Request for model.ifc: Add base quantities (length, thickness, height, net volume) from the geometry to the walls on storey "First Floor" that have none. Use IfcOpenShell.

First a look at what the model holds.

```python
import ifcopenshell
import ifcopenshell.util.element
import ifcopenshell.util.unit

model = ifcopenshell.open("model.ifc")
print(model.schema)
for unit_type in ("LENGTHUNIT", "AREAUNIT", "VOLUMEUNIT"):
    print(unit_type, ifcopenshell.util.unit.calculate_unit_scale(model, unit_type))
storey = next(s for s in model.by_type("IfcBuildingStorey") if s.Name == "First Floor")
walls = [e for e in ifcopenshell.util.element.get_decomposition(storey) if e.is_a("IfcWall")]
for e in sorted(walls, key=lambda e: e.id()):
    print(e.id(), e.is_a(), e.Name, list(ifcopenshell.util.element.get_psets(e, qtos_only=True)), sep=" | ")
```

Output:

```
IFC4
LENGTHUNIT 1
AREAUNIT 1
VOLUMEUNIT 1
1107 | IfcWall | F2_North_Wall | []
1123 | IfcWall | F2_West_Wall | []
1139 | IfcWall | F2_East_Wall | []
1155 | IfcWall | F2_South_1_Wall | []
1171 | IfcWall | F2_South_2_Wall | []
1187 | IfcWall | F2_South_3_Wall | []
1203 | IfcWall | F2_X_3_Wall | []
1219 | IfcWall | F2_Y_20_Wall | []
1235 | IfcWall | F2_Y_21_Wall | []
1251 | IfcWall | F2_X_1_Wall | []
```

```python
import ifcopenshell
import ifcopenshell.api.pset
import ifcopenshell.geom
import ifcopenshell.util.element
import ifcopenshell.util.shape
import ifcopenshell.util.unit

model = ifcopenshell.open("model.ifc")
unit_scale = ifcopenshell.util.unit.calculate_unit_scale(model)
volume_scale = ifcopenshell.util.unit.calculate_unit_scale(model, "VOLUMEUNIT")
settings = ifcopenshell.geom.settings()

storey = next(s for s in model.by_type("IfcBuildingStorey") if s.Name == "First Floor")
walls = [e for e in ifcopenshell.util.element.get_decomposition(storey) if e.is_a("IfcWall")]

for e in sorted(walls, key=lambda e: e.id()):
    if ifcopenshell.util.element.get_psets(e, qtos_only=True, should_inherit=False):
        continue
    # Geometry comes back in metres, in the element's own axes.
    shape = ifcopenshell.geom.create_shape(settings, e)
    values = {
        "Length": ifcopenshell.util.shape.get_x(shape.geometry) / unit_scale,
        "Width": ifcopenshell.util.shape.get_y(shape.geometry) / unit_scale,
        "Height": ifcopenshell.util.shape.get_z(shape.geometry) / unit_scale,
        "NetVolume": ifcopenshell.util.shape.get_volume(shape.geometry) / volume_scale,
    }
    qto = ifcopenshell.api.pset.add_qto(model, product=e, name="Qto_WallBaseQuantities")
    ifcopenshell.api.pset.edit_qto(model, qto=qto, properties=values)
    print(e.id(), {k: round(v, 3) for k, v in values.items()})

model.write("model_rev.ifc")
```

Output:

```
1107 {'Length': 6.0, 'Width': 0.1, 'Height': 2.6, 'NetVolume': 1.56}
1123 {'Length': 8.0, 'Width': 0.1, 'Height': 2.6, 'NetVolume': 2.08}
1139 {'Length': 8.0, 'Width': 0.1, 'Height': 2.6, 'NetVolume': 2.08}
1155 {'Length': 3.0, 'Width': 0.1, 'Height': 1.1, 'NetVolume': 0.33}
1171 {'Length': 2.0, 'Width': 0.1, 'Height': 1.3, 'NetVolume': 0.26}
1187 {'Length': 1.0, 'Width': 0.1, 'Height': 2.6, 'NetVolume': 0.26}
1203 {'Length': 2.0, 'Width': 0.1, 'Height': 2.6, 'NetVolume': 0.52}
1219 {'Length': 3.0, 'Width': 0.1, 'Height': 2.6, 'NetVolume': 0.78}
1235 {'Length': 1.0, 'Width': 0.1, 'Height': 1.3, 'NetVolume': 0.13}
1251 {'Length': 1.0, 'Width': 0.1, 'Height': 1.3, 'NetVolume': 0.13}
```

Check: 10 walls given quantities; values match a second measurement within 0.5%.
